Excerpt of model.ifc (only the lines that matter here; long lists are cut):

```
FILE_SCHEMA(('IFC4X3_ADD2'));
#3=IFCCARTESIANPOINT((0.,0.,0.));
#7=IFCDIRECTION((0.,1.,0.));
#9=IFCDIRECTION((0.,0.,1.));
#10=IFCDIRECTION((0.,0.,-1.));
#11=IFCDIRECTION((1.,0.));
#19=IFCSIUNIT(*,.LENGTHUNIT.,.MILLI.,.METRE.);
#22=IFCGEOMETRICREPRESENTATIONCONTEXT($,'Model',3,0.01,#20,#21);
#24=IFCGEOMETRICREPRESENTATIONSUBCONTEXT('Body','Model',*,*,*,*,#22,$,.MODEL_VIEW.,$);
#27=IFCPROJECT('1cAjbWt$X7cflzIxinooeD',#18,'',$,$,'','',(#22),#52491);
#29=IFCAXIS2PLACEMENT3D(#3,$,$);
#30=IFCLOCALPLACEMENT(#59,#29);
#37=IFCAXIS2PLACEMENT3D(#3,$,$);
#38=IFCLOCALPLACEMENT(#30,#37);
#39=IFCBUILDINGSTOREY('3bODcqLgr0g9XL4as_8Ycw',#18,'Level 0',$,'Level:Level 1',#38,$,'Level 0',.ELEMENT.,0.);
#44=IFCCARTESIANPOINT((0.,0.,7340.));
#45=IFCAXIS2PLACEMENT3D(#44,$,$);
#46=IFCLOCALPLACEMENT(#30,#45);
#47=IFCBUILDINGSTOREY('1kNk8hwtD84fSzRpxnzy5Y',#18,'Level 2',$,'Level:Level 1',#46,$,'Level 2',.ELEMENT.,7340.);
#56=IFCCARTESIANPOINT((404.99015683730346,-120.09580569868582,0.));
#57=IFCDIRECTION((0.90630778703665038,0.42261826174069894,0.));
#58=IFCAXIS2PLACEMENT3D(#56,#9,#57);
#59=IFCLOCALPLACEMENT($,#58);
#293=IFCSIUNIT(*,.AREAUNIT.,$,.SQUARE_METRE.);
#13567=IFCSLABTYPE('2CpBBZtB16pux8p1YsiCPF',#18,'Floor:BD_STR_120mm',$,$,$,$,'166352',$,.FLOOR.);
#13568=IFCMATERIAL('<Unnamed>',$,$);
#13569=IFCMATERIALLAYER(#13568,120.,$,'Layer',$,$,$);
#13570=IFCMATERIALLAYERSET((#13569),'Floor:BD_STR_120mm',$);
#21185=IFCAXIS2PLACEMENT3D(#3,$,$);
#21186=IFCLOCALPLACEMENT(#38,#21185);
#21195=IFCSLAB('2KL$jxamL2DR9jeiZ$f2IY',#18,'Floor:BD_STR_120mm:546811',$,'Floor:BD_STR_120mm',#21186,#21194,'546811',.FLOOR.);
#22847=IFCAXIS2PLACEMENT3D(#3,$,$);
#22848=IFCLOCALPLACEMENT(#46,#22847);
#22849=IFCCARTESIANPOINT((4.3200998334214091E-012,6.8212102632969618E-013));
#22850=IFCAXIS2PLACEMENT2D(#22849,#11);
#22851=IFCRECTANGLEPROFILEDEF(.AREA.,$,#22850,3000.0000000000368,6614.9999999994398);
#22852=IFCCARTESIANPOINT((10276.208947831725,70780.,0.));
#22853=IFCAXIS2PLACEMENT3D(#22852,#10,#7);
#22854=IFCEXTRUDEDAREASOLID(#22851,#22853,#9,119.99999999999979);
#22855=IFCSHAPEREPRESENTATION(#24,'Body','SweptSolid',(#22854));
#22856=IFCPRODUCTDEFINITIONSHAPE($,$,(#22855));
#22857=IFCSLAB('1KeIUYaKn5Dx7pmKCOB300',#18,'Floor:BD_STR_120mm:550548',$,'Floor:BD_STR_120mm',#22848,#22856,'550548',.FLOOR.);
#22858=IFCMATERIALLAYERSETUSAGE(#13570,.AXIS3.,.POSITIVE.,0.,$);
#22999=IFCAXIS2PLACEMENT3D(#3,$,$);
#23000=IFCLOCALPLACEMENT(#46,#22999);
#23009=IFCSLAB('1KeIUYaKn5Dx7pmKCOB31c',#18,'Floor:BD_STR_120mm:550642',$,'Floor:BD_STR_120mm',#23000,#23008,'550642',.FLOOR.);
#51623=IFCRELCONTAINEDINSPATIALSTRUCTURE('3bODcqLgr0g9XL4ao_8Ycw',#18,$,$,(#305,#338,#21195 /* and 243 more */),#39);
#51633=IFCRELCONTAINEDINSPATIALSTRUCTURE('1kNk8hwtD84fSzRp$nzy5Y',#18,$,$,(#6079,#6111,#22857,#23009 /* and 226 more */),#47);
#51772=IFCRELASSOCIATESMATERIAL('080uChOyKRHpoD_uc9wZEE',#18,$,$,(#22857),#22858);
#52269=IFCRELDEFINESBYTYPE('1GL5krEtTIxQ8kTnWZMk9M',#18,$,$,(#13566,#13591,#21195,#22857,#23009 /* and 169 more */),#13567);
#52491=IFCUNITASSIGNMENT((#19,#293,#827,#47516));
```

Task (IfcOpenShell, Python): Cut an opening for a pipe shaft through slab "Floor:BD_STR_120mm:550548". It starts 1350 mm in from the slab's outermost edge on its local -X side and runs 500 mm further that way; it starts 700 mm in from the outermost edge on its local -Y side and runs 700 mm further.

```python
import numpy as np
import ifcopenshell
import ifcopenshell.api.feature
import ifcopenshell.api.geometry
import ifcopenshell.api.root
import ifcopenshell.geom
import ifcopenshell.util.placement
import ifcopenshell.util.representation
import ifcopenshell.util.shape
import ifcopenshell.util.unit

model = ifcopenshell.open("model.ifc")
unit_scale = ifcopenshell.util.unit.calculate_unit_scale(model)
settings = ifcopenshell.geom.settings()


def volume(element):
    """Net volume in cubic metres, openings subtracted."""
    shape = ifcopenshell.geom.create_shape(settings, element)
    return ifcopenshell.util.shape.get_volume(shape.geometry)


slab = model.by_guid("1KeIUYaKn5Dx7pmKCOB300")
before = volume(slab)

# Extent in the slab's own axes, in metres. The edges named are its -X and -Y sides.
slab_shape = ifcopenshell.geom.create_shape(settings, slab)
vertices = ifcopenshell.util.shape.get_vertices(slab_shape.geometry)
x_min, y_min, bottom = vertices.min(axis=0)
top = vertices[:, 2].max()

opening = ifcopenshell.api.root.create_entity(model, ifc_class="IfcOpeningElement", name="Pipe shaft opening", predefined_type="OPENING")
context = ifcopenshell.util.representation.get_context(model, "Model", "Body", "MODEL_VIEW")
width, depth = 0.5, 0.7
outline = [(0.0, 0.0), (width, 0.0), (width, depth), (0.0, depth), (0.0, 0.0)]
# Overshoot both faces by 50 mm so the cut is clean.
shape = ifcopenshell.api.geometry.add_slab_representation(
    model, context=context, depth=top - bottom + 0.1, polyline=outline
)
ifcopenshell.api.geometry.assign_representation(model, product=opening, representation=shape)

matrix = ifcopenshell.util.placement.get_local_placement(slab.ObjectPlacement)
matrix[:, 3] = matrix @ np.append(np.array([x_min + 1.35, y_min + 0.7, bottom - 0.05]) / unit_scale, 1.0)
ifcopenshell.api.geometry.edit_object_placement(model, product=opening, matrix=matrix, is_si=False)
ifcopenshell.api.feature.add_feature(model, feature=opening, element=slab)

after = volume(slab)

print(f"slab volume {before:.3f} -> {after:.3f} m3")

model.write("model-out.ifc")
```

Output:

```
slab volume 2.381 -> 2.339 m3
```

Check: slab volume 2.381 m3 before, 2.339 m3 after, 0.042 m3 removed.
